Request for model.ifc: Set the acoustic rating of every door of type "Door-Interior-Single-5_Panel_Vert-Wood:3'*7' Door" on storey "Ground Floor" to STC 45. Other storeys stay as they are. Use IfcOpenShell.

First a look at what the model holds.

```python
import ifcopenshell
import ifcopenshell.util.element

model = ifcopenshell.open("model.ifc")
print(model.schema)
storey = next(s for s in model.by_type("IfcBuildingStorey") if s.Name == "Ground Floor")
doors = [e for e in ifcopenshell.util.element.get_decomposition(storey) if e.is_a("IfcDoor")]
seen = {}
for e in doors:
    element_type = ifcopenshell.util.element.get_type(e)
    key = (element_type.Name if element_type != e and element_type else None, ifcopenshell.util.element.get_pset(e, "Pset_DoorCommon", "AcousticRating"))
    seen[key] = seen.get(key, 0) + 1
for (name, value), count in sorted(seen.items(), key=str):
    print(count, "x", name, "|", value)
```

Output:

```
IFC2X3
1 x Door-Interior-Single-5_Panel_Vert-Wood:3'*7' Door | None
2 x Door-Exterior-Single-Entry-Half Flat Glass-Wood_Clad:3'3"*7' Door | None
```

```python
import ifcopenshell
import ifcopenshell.api.pset
import ifcopenshell.util.element

model = ifcopenshell.open("model.ifc")

storey = next(s for s in model.by_type("IfcBuildingStorey") if s.Name == "Ground Floor")
doors = [e for e in ifcopenshell.util.element.get_decomposition(storey) if e.is_a("IfcDoor")]

count = 0
for e in doors:
    element_type = ifcopenshell.util.element.get_type(e)
    if element_type in (None, e) or element_type.Name != "Door-Interior-Single-5_Panel_Vert-Wood:3'*7' Door":
        continue
    # add_pset returns the element's existing set when there is one.
    pset = ifcopenshell.api.pset.add_pset(model, product=e, name="Pset_DoorCommon")
    ifcopenshell.api.pset.edit_pset(model, pset=pset, properties={"AcousticRating": "STC 45"})
    count += 1

print(count, "doors updated")

model.write("model_rev.ifc")
```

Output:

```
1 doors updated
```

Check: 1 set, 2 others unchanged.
